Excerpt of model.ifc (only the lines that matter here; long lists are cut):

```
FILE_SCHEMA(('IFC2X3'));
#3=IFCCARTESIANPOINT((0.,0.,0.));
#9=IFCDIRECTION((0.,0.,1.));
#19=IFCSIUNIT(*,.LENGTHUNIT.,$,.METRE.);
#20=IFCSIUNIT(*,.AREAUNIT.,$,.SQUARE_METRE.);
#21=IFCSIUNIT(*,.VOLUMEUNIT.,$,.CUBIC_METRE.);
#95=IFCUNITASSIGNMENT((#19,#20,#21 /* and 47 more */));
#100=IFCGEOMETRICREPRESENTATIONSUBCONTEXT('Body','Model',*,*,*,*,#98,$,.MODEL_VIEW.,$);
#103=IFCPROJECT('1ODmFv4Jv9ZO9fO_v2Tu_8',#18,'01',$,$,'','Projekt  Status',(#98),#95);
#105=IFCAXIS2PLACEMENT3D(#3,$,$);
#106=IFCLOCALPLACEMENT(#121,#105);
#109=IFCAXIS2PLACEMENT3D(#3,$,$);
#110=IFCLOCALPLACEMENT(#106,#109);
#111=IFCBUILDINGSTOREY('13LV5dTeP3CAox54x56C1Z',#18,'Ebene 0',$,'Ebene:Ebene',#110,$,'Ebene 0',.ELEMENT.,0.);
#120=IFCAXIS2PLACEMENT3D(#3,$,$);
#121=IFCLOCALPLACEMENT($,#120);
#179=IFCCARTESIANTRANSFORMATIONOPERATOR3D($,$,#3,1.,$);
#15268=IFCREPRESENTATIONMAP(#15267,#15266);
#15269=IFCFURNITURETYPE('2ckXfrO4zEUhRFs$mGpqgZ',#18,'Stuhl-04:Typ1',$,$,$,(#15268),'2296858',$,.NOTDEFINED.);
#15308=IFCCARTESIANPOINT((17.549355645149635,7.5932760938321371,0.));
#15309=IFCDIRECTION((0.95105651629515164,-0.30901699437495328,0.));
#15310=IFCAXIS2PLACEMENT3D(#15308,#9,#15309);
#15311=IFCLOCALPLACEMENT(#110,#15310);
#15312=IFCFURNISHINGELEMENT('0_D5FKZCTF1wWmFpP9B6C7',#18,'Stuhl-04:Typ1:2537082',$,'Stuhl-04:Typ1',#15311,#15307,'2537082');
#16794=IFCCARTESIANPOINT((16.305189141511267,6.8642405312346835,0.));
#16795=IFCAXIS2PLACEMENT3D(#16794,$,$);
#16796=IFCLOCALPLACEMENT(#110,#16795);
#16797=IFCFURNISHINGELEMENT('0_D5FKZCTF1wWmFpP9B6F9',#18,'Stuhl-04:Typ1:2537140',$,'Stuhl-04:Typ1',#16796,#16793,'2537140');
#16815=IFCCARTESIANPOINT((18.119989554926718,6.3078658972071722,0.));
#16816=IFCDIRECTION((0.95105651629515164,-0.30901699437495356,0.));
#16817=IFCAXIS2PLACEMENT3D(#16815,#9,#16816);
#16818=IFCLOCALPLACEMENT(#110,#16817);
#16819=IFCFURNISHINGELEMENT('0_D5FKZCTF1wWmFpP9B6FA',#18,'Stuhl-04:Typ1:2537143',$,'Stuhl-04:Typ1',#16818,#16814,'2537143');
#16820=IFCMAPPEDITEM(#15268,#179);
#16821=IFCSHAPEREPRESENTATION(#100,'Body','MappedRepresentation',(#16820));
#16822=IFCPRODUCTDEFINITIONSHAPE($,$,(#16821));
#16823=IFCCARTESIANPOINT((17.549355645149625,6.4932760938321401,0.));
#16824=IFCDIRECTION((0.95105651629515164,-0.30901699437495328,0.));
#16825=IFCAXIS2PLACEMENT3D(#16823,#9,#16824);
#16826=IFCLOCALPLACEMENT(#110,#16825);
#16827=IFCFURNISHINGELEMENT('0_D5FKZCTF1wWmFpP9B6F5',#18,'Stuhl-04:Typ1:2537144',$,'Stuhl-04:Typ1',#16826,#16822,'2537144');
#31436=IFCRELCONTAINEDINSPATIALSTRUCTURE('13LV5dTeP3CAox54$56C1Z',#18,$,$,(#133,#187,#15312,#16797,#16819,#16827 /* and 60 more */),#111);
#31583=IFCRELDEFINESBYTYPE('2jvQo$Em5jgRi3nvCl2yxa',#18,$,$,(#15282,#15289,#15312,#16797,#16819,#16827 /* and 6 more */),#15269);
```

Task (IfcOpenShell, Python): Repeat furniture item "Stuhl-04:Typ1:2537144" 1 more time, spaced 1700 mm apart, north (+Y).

```python
import numpy as np
import ifcopenshell
import ifcopenshell.api.geometry
import ifcopenshell.api.root
import ifcopenshell.util.element
import ifcopenshell.util.placement
import ifcopenshell.util.unit

model = ifcopenshell.open("model.ifc")
unit_scale = ifcopenshell.util.unit.calculate_unit_scale(model)

source = model.by_guid("0_D5FKZCTF1wWmFpP9B6F5")
base = ifcopenshell.util.placement.get_local_placement(source.ObjectPlacement)
step = np.array([0.0, 1.0, 0.0]) * 1.7 / unit_scale

for i in range(1, 2):
    copy = ifcopenshell.api.root.copy_class(model, product=source)
    copy.Representation = ifcopenshell.util.element.copy_deep(
        model, source.Representation, exclude=["IfcGeometricRepresentationContext", "IfcRepresentationMap"]
    )
    copy.Name = "Stuhl-04:Typ1"
    copy.Tag = None
    matrix = base.copy()
    matrix[:3, 3] += i * step
    print("added at", matrix[:3, 3].round(3) + 0.0)
    ifcopenshell.api.geometry.edit_object_placement(model, product=copy, matrix=matrix, is_si=False)

model.write("model_rev.ifc")
```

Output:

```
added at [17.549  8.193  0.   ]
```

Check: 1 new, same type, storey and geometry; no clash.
